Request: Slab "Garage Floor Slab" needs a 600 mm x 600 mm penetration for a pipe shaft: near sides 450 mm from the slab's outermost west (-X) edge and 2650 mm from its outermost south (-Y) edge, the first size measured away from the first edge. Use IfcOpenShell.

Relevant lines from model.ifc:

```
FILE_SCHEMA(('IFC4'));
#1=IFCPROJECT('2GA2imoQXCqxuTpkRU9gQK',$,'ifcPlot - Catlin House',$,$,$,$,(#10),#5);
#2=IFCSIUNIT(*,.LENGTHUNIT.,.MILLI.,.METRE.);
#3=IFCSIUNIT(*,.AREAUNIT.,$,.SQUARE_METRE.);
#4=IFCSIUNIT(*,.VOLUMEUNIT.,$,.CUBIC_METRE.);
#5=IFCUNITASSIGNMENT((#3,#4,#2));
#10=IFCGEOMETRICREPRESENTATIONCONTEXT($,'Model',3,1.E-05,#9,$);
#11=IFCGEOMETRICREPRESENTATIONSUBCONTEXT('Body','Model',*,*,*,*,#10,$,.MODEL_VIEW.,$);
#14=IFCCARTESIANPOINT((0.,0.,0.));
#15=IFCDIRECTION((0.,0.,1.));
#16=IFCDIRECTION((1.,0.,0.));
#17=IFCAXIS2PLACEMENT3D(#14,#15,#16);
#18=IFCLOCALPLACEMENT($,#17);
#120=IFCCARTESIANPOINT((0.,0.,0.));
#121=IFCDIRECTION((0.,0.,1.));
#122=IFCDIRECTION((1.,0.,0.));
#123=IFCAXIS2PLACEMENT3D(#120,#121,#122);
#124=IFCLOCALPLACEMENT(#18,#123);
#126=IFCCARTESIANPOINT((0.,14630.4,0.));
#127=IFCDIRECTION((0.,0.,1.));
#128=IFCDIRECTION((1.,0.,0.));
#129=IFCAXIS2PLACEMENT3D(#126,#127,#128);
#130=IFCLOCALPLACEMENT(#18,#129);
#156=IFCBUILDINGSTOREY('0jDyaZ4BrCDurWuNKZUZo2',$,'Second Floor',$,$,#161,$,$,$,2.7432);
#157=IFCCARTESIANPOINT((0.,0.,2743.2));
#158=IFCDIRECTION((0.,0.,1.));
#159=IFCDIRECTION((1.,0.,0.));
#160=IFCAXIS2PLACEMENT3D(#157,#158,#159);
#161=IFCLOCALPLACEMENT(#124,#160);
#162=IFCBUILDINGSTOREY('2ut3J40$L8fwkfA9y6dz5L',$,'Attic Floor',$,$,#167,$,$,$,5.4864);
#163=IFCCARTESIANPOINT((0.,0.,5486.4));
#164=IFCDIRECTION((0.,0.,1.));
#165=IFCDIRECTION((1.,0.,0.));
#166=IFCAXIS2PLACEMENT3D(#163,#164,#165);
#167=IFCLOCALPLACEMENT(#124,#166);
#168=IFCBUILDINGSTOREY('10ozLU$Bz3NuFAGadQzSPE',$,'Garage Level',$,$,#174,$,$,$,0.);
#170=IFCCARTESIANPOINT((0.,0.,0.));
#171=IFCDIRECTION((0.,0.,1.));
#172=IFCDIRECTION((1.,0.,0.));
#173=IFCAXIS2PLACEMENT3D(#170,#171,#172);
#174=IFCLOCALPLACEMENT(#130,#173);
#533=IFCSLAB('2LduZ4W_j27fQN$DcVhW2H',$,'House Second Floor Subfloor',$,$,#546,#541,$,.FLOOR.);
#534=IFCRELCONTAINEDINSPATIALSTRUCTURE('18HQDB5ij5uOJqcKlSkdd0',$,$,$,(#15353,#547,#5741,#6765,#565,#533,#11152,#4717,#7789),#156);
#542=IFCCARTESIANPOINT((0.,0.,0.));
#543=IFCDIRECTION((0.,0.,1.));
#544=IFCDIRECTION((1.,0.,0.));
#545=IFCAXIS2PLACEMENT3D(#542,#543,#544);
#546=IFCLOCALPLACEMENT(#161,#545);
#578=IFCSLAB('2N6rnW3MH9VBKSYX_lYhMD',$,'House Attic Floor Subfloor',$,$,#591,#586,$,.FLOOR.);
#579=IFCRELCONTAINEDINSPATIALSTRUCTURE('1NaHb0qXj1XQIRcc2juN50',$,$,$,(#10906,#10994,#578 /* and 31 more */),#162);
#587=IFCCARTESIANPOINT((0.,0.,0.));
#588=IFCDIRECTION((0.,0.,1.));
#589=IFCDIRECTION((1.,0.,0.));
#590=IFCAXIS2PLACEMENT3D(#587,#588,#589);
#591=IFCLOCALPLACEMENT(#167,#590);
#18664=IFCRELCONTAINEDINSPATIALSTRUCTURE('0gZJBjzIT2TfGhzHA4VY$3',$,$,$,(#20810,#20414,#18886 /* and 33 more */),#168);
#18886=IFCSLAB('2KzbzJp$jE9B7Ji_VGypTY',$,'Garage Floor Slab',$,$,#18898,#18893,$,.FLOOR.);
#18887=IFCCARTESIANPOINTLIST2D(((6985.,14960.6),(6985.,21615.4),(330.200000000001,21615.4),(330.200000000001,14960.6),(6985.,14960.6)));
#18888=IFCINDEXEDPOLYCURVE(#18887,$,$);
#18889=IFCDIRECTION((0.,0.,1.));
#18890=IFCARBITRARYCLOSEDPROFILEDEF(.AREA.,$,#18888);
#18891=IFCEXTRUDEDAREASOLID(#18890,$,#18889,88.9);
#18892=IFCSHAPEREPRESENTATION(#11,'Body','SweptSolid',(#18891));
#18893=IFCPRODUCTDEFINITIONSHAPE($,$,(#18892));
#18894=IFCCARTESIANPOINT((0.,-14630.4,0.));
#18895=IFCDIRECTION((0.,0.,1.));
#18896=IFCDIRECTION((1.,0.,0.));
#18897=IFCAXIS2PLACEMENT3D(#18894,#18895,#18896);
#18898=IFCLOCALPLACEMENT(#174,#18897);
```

```python
import numpy as np
import ifcopenshell
import ifcopenshell.api.feature
import ifcopenshell.api.geometry
import ifcopenshell.api.root
import ifcopenshell.geom
import ifcopenshell.util.placement
import ifcopenshell.util.representation
import ifcopenshell.util.shape
import ifcopenshell.util.unit

model = ifcopenshell.open("model.ifc")
unit_scale = ifcopenshell.util.unit.calculate_unit_scale(model)
settings = ifcopenshell.geom.settings()


def volume(element):
    """Net volume in cubic metres, openings subtracted."""
    shape = ifcopenshell.geom.create_shape(settings, element)
    return ifcopenshell.util.shape.get_volume(shape.geometry)


slab = model.by_guid("2KzbzJp$jE9B7Ji_VGypTY")
before = volume(slab)

# Extent in the slab's own axes, in metres. The edges named are its -X and -Y sides.
slab_shape = ifcopenshell.geom.create_shape(settings, slab)
vertices = ifcopenshell.util.shape.get_vertices(slab_shape.geometry)
x_min, y_min, bottom = vertices.min(axis=0)
top = vertices[:, 2].max()

opening = ifcopenshell.api.root.create_entity(model, ifc_class="IfcOpeningElement", name="Pipe shaft opening", predefined_type="OPENING")
context = ifcopenshell.util.representation.get_context(model, "Model", "Body", "MODEL_VIEW")
width, depth = 0.6, 0.6
outline = [(0.0, 0.0), (width, 0.0), (width, depth), (0.0, depth), (0.0, 0.0)]
# Overshoot both faces by 50 mm so the cut is clean.
shape = ifcopenshell.api.geometry.add_slab_representation(
    model, context=context, depth=top - bottom + 0.1, polyline=outline
)
ifcopenshell.api.geometry.assign_representation(model, product=opening, representation=shape)

matrix = ifcopenshell.util.placement.get_local_placement(slab.ObjectPlacement)
matrix[:, 3] = matrix @ np.append(np.array([x_min + 0.45, y_min + 2.65, bottom - 0.05]) / unit_scale, 1.0)
ifcopenshell.api.geometry.edit_object_placement(model, product=opening, matrix=matrix, is_si=False)
ifcopenshell.api.feature.add_feature(model, feature=opening, element=slab)

after = volume(slab)

print(f"slab volume {before:.3f} -> {after:.3f} m3")

model.write("model_edited.ifc")
```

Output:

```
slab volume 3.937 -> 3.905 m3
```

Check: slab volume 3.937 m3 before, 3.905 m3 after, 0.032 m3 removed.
